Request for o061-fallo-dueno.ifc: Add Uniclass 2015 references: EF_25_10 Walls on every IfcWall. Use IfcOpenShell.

First a look at what the model holds.

```python
import ifcopenshell

model = ifcopenshell.open("o061-fallo-dueno.ifc")
print(model.schema)
print("classifications:", [c.Name for c in model.by_type("IfcClassification")])
for ifc_class in ("IfcDoor", "IfcRoof", "IfcStair", "IfcWall", "IfcWindow"):
    print(ifc_class, len(model.by_type(ifc_class)))
```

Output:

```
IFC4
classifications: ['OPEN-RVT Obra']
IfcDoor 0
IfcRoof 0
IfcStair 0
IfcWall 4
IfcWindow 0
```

```python
import ifcopenshell
import ifcopenshell.api.classification

model = ifcopenshell.open("o061-fallo-dueno.ifc")

system = ifcopenshell.api.classification.add_classification(model, classification="Uniclass 2015")

codes = {
    "IfcWall": ("EF_25_10", "Walls"),
}
for ifc_class, (code, name) in codes.items():
    products = model.by_type(ifc_class)
    ifcopenshell.api.classification.add_reference(
        model, products=products, classification=system, identification=code, name=name
    )
    print(code, len(products))

model.write("o061-fallo-dueno_rev.ifc")
```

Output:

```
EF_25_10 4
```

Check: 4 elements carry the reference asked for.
